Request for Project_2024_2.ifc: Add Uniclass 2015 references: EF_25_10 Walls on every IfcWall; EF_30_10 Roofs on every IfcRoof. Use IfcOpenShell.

First a look at what the model holds.

```python
import ifcopenshell

model = ifcopenshell.open("Project_2024_2.ifc")
print(model.schema)
print("classifications:", [c.Name for c in model.by_type("IfcClassification")])
for ifc_class in ("IfcDoor", "IfcRoof", "IfcStair", "IfcWall", "IfcWindow"):
    print(ifc_class, len(model.by_type(ifc_class)))
```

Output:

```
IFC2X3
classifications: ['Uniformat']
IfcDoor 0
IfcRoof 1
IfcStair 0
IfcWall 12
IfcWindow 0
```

```python
import ifcopenshell
import ifcopenshell.api.classification

model = ifcopenshell.open("Project_2024_2.ifc")

# IFC2X3 requires Source and Edition and has no link from the project to the system.
system = model.create_entity("IfcClassification", Source="NBS", Edition="2015", Name="Uniclass 2015")

codes = {
    "IfcWall": ("EF_25_10", "Walls"),
    "IfcRoof": ("EF_30_10", "Roofs"),
}
for ifc_class, (code, name) in codes.items():
    products = model.by_type(ifc_class)
    ifcopenshell.api.classification.add_reference(
        model, products=products, classification=system, identification=code, name=name
    )
    print(code, len(products))

model.write("Project_2024_2_edited.ifc")
```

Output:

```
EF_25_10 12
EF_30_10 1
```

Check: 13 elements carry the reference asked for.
